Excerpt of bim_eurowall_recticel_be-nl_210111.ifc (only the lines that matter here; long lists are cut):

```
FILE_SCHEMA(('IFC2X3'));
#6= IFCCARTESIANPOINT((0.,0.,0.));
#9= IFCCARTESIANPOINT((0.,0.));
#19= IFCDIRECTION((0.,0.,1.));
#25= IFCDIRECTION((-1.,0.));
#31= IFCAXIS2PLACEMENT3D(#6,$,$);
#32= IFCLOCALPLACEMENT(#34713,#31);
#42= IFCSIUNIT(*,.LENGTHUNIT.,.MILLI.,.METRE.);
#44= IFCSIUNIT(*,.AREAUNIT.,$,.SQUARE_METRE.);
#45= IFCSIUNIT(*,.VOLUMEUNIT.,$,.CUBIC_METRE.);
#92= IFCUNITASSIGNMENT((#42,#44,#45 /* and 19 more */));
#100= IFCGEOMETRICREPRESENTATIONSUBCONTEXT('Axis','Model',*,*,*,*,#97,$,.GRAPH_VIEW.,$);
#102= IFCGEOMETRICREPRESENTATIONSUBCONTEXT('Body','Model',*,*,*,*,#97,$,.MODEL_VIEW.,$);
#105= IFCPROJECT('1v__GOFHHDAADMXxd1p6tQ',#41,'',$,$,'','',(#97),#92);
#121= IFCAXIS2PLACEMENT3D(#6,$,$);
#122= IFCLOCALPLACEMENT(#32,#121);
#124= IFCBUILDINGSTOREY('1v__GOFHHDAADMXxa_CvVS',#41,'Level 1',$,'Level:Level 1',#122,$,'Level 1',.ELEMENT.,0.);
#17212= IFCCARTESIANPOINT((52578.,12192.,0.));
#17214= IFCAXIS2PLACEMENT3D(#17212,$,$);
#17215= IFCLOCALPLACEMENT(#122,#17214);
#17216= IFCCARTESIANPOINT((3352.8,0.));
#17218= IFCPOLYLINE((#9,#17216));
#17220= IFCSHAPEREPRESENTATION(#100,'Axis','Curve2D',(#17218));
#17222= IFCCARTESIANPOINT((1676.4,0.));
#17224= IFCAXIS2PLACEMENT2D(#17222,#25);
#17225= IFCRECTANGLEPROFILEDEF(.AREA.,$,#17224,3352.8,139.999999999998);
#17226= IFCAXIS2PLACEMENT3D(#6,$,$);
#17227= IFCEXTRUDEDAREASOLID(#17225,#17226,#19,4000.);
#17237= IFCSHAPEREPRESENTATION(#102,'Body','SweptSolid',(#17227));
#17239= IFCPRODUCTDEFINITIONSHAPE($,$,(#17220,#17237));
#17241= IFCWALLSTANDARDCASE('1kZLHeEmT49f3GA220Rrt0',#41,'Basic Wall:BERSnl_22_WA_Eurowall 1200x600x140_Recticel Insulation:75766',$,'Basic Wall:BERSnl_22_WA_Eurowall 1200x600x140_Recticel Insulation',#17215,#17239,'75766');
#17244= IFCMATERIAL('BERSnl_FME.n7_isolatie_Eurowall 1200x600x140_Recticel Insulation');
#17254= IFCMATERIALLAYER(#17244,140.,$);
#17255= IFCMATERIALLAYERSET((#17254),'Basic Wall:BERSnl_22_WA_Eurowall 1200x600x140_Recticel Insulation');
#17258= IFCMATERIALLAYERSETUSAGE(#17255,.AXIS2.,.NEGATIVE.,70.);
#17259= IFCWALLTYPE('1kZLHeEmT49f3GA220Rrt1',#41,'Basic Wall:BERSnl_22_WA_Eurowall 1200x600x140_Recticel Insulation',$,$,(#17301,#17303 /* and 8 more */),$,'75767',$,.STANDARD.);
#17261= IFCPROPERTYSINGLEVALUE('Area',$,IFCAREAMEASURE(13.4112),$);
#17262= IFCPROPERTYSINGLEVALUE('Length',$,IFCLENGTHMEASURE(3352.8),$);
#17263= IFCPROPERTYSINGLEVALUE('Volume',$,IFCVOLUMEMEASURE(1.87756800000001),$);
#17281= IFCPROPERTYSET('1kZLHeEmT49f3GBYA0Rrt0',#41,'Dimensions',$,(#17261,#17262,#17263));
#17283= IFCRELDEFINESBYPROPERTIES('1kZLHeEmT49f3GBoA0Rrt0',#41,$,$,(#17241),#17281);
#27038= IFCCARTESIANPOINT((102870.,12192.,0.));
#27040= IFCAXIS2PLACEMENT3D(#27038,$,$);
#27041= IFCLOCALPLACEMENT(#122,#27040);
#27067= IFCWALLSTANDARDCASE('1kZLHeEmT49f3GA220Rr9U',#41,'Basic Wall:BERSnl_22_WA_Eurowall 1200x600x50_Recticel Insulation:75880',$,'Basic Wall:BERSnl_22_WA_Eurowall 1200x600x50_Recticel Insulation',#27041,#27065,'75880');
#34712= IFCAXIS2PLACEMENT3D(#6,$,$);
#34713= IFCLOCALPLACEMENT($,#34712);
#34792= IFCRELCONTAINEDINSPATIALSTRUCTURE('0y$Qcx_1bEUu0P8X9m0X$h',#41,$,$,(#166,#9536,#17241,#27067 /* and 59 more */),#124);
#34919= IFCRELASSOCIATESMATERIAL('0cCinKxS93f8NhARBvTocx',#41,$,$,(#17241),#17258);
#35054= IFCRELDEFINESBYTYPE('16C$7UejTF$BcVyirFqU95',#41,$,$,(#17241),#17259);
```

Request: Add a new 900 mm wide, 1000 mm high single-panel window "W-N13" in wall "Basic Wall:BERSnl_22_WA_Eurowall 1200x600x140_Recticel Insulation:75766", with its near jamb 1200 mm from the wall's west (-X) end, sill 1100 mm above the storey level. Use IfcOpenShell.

```python
import numpy as np
import ifcopenshell
import ifcopenshell.api.feature
import ifcopenshell.api.geometry
import ifcopenshell.api.pset
import ifcopenshell.api.root
import ifcopenshell.api.spatial
import ifcopenshell.api.type
import ifcopenshell.geom
import ifcopenshell.util.element
import ifcopenshell.util.placement
import ifcopenshell.util.representation
import ifcopenshell.util.shape
import ifcopenshell.util.unit

model = ifcopenshell.open("bim_eurowall_recticel_be-nl_210111.ifc")
unit_scale = ifcopenshell.util.unit.calculate_unit_scale(model)
area_scale = ifcopenshell.util.unit.calculate_unit_scale(model, "AREAUNIT")
volume_scale = ifcopenshell.util.unit.calculate_unit_scale(model, "VOLUMEUNIT")
settings = ifcopenshell.geom.settings()


def volume(element):
    """Net volume in cubic metres, openings subtracted."""
    shape = ifcopenshell.geom.create_shape(settings, element)
    return ifcopenshell.util.shape.get_volume(shape.geometry)


wall = model.by_guid("1kZLHeEmT49f3GA220Rrt0")
storey = ifcopenshell.util.element.get_container(wall, ifc_class="IfcBuildingStorey")
context = ifcopenshell.util.representation.get_context(model, "Model", "Body", "MODEL_VIEW")
before = volume(wall)

width, height, from_end, sill = 0.9, 1, 1.2, 1.1  # metres

# The wall runs along its own X axis, and the end named is its -X end.
wall_shape = ifcopenshell.geom.create_shape(settings, wall)
x, y, z = ifcopenshell.util.shape.get_vertices(wall_shape.geometry).T
start = x.min() + from_end
face, thickness = float(y.min()), float(y.max() - y.min())
wall_matrix = ifcopenshell.util.placement.get_local_placement(wall.ObjectPlacement)
level = ifcopenshell.util.placement.get_local_placement(storey.ObjectPlacement)[2, 3]


def in_wall(x, y):
    """Placement at x, y metres in the wall's axes, at sill height."""
    matrix = wall_matrix.copy()
    matrix[:, 3] = wall_matrix @ np.array([x / unit_scale, y / unit_scale, 0.0, 1.0])
    matrix[2, 3] = level + sill / unit_scale
    return matrix


# Opening: a box that overshoots both wall faces by 50 mm.
opening = ifcopenshell.api.root.create_entity(model, ifc_class="IfcOpeningElement")
box = ifcopenshell.api.geometry.add_wall_representation(
    model, context=context, length=width, height=height, thickness=thickness + 0.1
)
ifcopenshell.api.geometry.assign_representation(model, product=opening, representation=box)
ifcopenshell.api.geometry.edit_object_placement(model, product=opening, matrix=in_wall(start, face - 0.05), is_si=False)
ifcopenshell.api.feature.add_feature(model, feature=opening, element=wall)

window = ifcopenshell.api.root.create_entity(model, ifc_class="IfcWindow", name="W-N13")
window.OverallWidth, window.OverallHeight = width / unit_scale, height / unit_scale
body = ifcopenshell.api.geometry.add_window_representation(
    model,
    context=context,
    overall_width=window.OverallWidth,
    overall_height=window.OverallHeight,
    partition_type="SINGLE_PANEL",
)
ifcopenshell.api.geometry.assign_representation(model, product=window, representation=body)
ifcopenshell.api.spatial.assign_container(model, products=[window], relating_structure=storey)
fills = ifcopenshell.api.feature.add_filling(model, opening=opening, element=window)
fills.OwnerHistory = window.OwnerHistory  # required in IFC2X3

# IFC2X3 keeps the operation on the window style.
style = ifcopenshell.api.root.create_entity(model, ifc_class="IfcWindowStyle", name="W-N13")
style.OperationType, style.ConstructionType = "SINGLE_PANEL", "NOTDEFINED"
style.ParameterTakesPrecedence = style.Sizeable = False
ifcopenshell.api.type.assign_type(model, related_objects=[window], relating_type=style)

# Centre the window in the wall's thickness.
ifcopenshell.api.geometry.edit_object_placement(model, product=window, matrix=in_wall(start, face), is_si=False)
window_shape = ifcopenshell.geom.create_shape(settings, window)
depth = ifcopenshell.util.shape.get_vertices(window_shape.geometry)[:, 1]
offset = face + thickness / 2 - (depth.min() + depth.max()) / 2
ifcopenshell.api.geometry.edit_object_placement(model, product=window, matrix=in_wall(start, offset), is_si=False)

after = volume(wall)

# Update the wall's stored quantities.
pset = model.by_id(ifcopenshell.util.element.get_pset(wall, "Dimensions", should_inherit=False)["id"])
ifcopenshell.api.pset.edit_pset(model, pset=pset, properties={
    "Area": model.create_entity("IfcAreaMeasure", after / thickness / area_scale),
    "Volume": model.create_entity("IfcVolumeMeasure", after / volume_scale),
})

print(f"wall volume {before:.3f} -> {after:.3f} m3")

model.write("bim_eurowall_recticel_be-nl_210111_edited.ifc")
```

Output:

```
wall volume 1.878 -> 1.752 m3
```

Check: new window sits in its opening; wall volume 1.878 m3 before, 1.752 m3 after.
